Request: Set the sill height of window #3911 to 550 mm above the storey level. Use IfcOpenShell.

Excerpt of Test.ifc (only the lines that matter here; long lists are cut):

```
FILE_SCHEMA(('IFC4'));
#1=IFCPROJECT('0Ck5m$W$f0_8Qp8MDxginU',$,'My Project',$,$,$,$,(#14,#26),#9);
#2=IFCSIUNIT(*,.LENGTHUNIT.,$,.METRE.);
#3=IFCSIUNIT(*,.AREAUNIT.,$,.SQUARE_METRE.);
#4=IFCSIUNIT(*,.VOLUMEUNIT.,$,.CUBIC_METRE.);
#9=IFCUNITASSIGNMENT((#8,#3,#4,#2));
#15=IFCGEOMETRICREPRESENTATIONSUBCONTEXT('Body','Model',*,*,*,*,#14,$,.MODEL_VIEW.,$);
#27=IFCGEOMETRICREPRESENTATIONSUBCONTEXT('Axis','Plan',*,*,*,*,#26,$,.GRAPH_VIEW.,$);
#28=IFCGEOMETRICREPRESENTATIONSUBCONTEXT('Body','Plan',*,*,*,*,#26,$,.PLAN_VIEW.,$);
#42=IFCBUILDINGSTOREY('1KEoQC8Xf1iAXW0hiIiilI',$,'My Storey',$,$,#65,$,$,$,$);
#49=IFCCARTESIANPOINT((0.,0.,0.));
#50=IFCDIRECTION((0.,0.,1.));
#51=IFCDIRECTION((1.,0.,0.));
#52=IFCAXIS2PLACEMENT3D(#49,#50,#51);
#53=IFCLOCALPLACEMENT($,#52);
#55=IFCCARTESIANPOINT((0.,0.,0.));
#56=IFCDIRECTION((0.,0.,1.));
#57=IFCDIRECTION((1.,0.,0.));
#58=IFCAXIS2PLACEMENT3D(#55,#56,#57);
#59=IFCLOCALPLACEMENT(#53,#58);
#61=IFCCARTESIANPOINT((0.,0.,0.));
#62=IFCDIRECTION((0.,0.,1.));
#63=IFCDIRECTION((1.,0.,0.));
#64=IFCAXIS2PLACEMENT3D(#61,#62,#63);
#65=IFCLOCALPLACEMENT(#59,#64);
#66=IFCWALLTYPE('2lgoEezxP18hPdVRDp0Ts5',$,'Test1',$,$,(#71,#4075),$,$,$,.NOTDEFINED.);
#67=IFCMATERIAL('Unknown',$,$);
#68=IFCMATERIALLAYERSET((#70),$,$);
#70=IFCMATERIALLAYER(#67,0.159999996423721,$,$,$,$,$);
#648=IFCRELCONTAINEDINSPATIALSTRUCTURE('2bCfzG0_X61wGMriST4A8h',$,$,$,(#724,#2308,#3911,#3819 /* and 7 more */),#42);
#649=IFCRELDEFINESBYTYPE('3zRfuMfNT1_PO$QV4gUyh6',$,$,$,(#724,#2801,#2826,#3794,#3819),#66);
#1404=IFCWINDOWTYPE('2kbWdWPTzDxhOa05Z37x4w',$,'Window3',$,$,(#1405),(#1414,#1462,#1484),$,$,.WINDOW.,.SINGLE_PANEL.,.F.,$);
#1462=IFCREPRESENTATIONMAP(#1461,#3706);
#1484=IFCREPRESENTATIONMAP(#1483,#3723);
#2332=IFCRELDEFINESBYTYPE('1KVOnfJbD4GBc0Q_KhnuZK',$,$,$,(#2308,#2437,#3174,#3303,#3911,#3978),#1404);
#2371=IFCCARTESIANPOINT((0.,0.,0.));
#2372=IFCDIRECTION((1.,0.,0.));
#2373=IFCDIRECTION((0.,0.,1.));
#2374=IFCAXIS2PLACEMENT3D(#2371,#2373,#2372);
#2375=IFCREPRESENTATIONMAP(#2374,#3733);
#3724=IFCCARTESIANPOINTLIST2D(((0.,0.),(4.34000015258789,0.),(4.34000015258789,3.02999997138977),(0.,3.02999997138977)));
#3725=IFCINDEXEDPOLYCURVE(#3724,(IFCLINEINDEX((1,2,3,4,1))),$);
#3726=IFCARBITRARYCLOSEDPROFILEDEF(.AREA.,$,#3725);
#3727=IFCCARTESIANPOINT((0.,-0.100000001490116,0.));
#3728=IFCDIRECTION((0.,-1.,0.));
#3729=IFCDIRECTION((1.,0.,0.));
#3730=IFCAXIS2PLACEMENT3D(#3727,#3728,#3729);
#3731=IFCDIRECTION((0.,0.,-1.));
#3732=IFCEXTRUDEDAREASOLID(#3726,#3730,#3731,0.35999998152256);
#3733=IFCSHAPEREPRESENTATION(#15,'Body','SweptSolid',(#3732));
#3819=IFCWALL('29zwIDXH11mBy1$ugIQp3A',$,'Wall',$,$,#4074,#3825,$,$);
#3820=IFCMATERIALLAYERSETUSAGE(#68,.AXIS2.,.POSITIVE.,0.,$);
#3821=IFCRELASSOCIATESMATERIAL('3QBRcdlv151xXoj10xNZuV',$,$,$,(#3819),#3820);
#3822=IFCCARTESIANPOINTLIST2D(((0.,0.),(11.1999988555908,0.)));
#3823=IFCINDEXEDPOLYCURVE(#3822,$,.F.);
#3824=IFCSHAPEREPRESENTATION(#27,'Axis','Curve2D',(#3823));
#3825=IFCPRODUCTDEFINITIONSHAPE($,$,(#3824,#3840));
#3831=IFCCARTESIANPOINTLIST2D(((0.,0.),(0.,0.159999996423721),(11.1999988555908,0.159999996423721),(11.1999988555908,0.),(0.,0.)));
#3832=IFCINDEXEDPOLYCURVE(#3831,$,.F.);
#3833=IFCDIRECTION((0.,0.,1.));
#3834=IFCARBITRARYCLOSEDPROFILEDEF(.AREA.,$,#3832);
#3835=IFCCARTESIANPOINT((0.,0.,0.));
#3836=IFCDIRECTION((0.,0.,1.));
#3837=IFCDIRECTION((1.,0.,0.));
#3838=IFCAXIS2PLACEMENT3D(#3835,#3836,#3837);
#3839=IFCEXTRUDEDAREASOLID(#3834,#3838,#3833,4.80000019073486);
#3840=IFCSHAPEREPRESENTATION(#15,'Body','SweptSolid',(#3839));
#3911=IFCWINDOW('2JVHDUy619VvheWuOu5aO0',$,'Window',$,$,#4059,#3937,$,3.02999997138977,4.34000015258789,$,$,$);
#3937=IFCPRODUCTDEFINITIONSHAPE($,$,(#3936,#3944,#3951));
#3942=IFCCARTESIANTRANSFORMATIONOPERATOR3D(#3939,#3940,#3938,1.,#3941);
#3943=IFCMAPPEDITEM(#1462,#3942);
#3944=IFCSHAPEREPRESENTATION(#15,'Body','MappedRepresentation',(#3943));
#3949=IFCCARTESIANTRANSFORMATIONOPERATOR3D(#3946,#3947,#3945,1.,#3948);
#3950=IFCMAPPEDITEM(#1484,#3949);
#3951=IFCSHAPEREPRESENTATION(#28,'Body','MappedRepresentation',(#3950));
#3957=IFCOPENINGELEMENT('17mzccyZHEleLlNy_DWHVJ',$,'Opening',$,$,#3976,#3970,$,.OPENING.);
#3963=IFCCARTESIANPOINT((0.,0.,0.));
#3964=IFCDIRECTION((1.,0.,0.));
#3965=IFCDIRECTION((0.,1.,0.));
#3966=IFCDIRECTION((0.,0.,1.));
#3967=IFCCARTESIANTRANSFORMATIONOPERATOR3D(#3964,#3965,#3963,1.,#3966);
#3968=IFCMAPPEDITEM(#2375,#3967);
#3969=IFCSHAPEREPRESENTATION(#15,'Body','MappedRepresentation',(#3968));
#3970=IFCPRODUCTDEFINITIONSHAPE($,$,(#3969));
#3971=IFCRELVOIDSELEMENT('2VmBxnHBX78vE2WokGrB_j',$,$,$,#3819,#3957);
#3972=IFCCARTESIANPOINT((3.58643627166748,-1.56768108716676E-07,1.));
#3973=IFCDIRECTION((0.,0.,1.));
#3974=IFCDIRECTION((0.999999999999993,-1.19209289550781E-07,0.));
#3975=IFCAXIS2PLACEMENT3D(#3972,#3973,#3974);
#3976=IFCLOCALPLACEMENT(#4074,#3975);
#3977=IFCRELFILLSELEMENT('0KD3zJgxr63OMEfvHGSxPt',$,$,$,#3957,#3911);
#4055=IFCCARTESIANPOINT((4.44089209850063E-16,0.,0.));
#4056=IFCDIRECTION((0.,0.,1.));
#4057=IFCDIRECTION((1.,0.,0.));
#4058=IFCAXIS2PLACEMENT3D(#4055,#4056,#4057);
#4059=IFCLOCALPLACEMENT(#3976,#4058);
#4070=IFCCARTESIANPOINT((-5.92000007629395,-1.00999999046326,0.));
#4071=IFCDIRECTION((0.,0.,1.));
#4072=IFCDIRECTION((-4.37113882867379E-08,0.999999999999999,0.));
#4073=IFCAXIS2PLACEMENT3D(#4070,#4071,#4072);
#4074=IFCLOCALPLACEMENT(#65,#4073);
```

```python
import numpy as np
import ifcopenshell
import ifcopenshell.api.geometry
import ifcopenshell.geom
import ifcopenshell.util.element
import ifcopenshell.util.placement
import ifcopenshell.util.shape
import ifcopenshell.util.unit

model = ifcopenshell.open("Test.ifc")
unit_scale = ifcopenshell.util.unit.calculate_unit_scale(model)

window = model.by_guid("2JVHDUy619VvheWuOu5aO0")
opening = window.FillsVoids[0].RelatingOpeningElement
storey = ifcopenshell.util.element.get_container(window, ifc_class="IfcBuildingStorey")
level = ifcopenshell.util.placement.get_local_placement(storey.ObjectPlacement)[2, 3]

# The opening's origin need not be at the sill, so measure its lowest point.
shape = ifcopenshell.geom.create_shape(ifcopenshell.geom.settings(), opening)
bottom = ifcopenshell.util.shape.get_shape_bottom_elevation(shape, shape.geometry) / unit_scale
dz = level + 0.55 - bottom

shift = np.array([0.0, 0.0, dz])
# The window is placed relative to its opening, so it follows when the opening moves.
matrix = ifcopenshell.util.placement.get_local_placement(opening.ObjectPlacement)
matrix[:3, 3] += shift
ifcopenshell.api.geometry.edit_object_placement(
    model, product=opening, matrix=matrix, is_si=False, should_transform_children=True
)

print(f"moved by {dz * unit_scale:+.3f} m")

model.write("Test_rev.ifc")
```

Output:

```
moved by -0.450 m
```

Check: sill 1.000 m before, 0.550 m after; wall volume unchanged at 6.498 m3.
